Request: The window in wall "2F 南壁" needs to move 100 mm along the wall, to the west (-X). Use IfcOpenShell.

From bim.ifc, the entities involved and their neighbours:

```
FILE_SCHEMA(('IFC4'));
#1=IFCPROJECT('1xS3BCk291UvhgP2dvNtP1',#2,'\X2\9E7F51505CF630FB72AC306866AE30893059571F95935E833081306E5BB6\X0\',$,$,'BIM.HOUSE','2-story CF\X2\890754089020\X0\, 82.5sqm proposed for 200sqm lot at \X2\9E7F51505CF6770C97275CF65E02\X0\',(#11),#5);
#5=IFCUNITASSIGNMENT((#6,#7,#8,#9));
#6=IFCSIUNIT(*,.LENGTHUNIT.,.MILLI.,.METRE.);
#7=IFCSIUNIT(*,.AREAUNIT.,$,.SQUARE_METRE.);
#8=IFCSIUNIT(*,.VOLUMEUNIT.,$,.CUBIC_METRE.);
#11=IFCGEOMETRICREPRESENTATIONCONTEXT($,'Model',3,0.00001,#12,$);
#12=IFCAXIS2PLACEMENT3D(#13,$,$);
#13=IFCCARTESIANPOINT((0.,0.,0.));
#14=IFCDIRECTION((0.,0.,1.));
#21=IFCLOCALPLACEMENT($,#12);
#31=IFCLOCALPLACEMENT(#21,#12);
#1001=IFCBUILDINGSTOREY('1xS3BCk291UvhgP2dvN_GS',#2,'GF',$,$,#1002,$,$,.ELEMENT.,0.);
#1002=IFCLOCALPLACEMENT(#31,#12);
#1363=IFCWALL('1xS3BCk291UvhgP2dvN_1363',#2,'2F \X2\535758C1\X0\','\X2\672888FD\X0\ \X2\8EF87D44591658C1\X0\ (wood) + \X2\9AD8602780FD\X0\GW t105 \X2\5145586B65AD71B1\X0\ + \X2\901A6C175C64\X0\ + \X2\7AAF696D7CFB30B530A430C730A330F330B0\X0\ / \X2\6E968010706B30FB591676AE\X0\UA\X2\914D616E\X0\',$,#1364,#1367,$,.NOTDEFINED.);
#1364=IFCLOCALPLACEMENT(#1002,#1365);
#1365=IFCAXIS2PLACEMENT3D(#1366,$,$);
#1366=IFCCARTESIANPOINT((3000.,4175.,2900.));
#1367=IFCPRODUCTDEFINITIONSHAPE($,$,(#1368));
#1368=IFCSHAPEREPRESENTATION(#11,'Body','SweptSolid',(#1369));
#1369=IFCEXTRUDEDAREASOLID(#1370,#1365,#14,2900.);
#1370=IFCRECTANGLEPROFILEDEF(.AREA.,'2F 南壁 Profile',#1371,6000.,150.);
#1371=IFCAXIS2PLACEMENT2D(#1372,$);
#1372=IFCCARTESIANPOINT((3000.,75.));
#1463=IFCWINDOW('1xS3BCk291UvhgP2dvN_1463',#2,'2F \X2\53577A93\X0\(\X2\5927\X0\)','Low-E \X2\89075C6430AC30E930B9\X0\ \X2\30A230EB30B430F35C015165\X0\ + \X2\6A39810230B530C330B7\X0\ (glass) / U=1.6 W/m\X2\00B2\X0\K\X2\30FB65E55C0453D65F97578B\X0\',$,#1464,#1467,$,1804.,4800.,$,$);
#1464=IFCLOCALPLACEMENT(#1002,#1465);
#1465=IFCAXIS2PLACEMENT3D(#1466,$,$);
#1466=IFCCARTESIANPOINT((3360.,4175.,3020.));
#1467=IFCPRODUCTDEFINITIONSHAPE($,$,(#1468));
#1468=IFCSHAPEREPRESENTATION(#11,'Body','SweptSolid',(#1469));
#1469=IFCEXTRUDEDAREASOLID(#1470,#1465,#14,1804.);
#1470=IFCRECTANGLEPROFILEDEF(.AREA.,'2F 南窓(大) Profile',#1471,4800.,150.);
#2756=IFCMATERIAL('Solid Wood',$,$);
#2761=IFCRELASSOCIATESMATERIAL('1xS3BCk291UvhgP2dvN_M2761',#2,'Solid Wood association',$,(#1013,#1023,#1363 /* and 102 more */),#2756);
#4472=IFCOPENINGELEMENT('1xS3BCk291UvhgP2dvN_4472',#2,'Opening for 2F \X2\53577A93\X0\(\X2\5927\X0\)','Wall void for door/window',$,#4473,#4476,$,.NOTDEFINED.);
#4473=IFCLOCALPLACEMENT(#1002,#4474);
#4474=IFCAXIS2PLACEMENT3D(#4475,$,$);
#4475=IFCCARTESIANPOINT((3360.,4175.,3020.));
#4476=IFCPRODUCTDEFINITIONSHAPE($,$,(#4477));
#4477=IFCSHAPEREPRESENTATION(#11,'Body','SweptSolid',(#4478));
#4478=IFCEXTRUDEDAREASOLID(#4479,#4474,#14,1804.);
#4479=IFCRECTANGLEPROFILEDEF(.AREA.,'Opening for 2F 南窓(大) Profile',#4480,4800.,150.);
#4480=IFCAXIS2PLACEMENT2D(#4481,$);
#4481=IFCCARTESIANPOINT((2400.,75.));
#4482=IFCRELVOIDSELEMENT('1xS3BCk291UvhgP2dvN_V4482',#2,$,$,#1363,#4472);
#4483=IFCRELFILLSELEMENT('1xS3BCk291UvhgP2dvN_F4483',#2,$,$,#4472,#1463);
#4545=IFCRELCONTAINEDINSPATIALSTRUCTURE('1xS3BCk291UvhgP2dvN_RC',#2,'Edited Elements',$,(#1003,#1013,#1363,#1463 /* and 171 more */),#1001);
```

```python
import ifcopenshell
import ifcopenshell.api.geometry
import ifcopenshell.util.placement

model = ifcopenshell.open("bim.ifc")

window = model.by_guid("1xS3BCk291UvhgP2dvN_1463")
opening = window.FillsVoids[0].RelatingOpeningElement
wall = opening.VoidsElements[0].RelatingBuildingElement

wall_matrix = ifcopenshell.util.placement.get_local_placement(wall.ObjectPlacement)
shift = wall_matrix[:3, 0] * -100.0
before = ifcopenshell.util.placement.get_local_placement(window.ObjectPlacement)[:3, 3].copy()

# The window is not placed relative to its opening, so move both.
for product in (opening, window):
    matrix = ifcopenshell.util.placement.get_local_placement(product.ObjectPlacement)
    matrix[:3, 3] += shift
    ifcopenshell.api.geometry.edit_object_placement(model, product=product, matrix=matrix, is_si=False)

after = ifcopenshell.util.placement.get_local_placement(window.ObjectPlacement)[:3, 3]
print("window moved by", (after - before).round(3) + 0.0)

model.write("bim_rev.ifc")
```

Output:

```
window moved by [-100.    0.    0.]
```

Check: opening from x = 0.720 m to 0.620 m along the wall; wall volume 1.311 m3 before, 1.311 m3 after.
